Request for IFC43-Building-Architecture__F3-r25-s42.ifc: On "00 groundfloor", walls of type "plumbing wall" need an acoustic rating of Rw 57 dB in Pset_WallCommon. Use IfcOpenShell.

First a look at what the model holds.

```python
import ifcopenshell
import ifcopenshell.util.element

model = ifcopenshell.open("IFC43-Building-Architecture__F3-r25-s42.ifc")
print(model.schema)
storey = next(s for s in model.by_type("IfcBuildingStorey") if s.Name == "00 groundfloor")
walls = [e for e in ifcopenshell.util.element.get_decomposition(storey) if e.is_a("IfcWall")]
seen = {}
for e in walls:
    element_type = ifcopenshell.util.element.get_type(e)
    key = (element_type.Name if element_type != e and element_type else None, ifcopenshell.util.element.get_pset(e, "Pset_WallCommon", "AcousticRating"))
    seen[key] = seen.get(key, 0) + 1
for (name, value), count in sorted(seen.items(), key=str):
    print(count, "x", name, "|", value)
```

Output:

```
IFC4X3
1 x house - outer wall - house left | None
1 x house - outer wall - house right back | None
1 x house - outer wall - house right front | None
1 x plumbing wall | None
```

```python
import ifcopenshell
import ifcopenshell.api.pset
import ifcopenshell.util.element

model = ifcopenshell.open("IFC43-Building-Architecture__F3-r25-s42.ifc")

storey = next(s for s in model.by_type("IfcBuildingStorey") if s.Name == "00 groundfloor")
walls = [e for e in ifcopenshell.util.element.get_decomposition(storey) if e.is_a("IfcWall")]

count = 0
for e in walls:
    element_type = ifcopenshell.util.element.get_type(e)
    if element_type in (None, e) or element_type.Name != "plumbing wall":
        continue
    # add_pset returns the element's existing set when there is one.
    pset = ifcopenshell.api.pset.add_pset(model, product=e, name="Pset_WallCommon")
    ifcopenshell.api.pset.edit_pset(model, pset=pset, properties={"AcousticRating": "Rw 57 dB"})
    count += 1

print(count, "walls updated")

model.write("IFC43-Building-Architecture__F3-r25-s42_updated.ifc")
```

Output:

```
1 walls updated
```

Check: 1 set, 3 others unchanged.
